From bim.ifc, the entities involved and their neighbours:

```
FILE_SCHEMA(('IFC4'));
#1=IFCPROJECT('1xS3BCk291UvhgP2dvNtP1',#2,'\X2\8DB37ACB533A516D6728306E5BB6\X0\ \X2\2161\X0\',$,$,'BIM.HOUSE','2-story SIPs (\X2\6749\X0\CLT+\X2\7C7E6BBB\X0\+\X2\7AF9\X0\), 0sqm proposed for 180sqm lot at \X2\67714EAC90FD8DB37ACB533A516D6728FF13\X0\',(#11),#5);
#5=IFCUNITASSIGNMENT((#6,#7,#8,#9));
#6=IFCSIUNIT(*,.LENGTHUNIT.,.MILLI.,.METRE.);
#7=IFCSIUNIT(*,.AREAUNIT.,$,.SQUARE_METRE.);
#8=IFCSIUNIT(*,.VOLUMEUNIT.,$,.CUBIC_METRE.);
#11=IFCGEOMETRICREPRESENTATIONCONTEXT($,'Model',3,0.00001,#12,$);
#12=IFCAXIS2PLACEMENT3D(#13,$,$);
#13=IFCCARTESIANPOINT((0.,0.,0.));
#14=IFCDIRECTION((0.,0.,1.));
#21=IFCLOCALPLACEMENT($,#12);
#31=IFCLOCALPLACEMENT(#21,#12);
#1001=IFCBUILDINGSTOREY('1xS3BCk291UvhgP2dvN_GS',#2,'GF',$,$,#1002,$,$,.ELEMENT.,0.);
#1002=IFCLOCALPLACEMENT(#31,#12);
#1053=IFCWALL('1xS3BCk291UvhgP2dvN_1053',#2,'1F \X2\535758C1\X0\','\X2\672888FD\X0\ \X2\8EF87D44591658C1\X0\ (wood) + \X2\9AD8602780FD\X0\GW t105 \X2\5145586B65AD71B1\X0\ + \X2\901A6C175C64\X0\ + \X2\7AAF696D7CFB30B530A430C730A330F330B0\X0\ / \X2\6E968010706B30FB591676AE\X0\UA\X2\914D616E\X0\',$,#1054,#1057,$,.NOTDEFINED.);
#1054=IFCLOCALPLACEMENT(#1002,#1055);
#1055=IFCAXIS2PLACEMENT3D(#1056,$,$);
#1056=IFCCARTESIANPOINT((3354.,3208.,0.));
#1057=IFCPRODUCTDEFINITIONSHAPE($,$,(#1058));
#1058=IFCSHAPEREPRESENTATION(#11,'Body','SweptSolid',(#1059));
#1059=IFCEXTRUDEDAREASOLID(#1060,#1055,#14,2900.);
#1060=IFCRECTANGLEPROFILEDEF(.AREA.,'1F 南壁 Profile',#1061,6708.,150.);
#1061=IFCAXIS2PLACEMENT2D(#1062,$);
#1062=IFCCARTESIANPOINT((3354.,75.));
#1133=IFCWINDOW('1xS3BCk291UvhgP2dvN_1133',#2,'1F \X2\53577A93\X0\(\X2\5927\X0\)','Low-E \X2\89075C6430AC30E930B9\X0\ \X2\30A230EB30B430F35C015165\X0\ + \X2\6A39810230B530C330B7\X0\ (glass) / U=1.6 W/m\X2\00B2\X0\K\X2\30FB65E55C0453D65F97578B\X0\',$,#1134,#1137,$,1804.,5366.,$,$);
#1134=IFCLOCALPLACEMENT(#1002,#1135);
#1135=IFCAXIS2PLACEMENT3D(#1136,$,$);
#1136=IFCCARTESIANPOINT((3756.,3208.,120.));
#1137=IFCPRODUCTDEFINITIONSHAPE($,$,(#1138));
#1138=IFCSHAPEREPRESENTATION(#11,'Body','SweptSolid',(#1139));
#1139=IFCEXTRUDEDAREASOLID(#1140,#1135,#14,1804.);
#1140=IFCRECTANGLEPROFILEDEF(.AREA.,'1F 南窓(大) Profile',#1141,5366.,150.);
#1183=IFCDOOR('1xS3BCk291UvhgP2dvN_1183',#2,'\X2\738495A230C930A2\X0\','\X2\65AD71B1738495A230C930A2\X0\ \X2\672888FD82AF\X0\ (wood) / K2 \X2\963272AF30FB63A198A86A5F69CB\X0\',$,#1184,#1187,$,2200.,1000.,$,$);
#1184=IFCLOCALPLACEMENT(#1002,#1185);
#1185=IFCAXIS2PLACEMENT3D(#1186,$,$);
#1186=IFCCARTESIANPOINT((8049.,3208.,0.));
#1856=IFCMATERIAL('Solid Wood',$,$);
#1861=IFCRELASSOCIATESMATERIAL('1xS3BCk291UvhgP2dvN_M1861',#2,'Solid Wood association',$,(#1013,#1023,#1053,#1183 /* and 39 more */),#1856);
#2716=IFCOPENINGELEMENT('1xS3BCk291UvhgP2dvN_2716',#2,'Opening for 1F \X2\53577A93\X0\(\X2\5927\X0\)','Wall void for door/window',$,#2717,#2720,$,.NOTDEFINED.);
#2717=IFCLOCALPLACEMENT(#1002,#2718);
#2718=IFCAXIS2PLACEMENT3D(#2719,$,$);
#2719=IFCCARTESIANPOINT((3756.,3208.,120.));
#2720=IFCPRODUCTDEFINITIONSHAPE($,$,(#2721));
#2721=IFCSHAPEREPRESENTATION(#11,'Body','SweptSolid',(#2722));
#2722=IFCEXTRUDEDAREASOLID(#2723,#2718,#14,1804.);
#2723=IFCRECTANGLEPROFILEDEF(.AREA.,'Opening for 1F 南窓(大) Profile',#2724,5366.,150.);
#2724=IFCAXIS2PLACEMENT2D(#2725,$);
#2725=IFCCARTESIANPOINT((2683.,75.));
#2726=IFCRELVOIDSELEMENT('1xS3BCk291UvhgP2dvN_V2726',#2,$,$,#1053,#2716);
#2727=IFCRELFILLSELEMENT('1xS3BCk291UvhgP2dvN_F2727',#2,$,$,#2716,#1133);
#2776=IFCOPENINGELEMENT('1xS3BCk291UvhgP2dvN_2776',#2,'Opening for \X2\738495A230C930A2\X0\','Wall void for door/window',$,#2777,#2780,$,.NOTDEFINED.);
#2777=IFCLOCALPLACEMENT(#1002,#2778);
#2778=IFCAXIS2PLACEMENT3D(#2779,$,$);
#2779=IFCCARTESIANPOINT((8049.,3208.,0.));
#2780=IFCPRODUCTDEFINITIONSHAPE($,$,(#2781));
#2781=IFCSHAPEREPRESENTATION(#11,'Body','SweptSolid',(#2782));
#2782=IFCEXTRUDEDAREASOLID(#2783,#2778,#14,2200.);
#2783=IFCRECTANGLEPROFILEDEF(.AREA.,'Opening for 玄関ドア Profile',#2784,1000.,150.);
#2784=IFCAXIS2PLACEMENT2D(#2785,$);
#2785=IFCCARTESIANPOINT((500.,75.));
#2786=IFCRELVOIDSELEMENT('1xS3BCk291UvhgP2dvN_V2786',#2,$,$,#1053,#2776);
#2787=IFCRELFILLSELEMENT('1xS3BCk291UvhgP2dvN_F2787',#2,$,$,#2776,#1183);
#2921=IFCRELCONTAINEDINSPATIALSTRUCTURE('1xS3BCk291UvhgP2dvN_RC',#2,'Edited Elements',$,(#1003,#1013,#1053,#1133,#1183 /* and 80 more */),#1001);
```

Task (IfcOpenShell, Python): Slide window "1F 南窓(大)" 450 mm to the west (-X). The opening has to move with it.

```python
import ifcopenshell
import ifcopenshell.api.geometry
import ifcopenshell.util.placement
import ifcopenshell.util.unit

model = ifcopenshell.open("bim.ifc")
unit_scale = ifcopenshell.util.unit.calculate_unit_scale(model)

window = model.by_guid("1xS3BCk291UvhgP2dvN_1133")
opening = window.FillsVoids[0].RelatingOpeningElement
wall = opening.VoidsElements[0].RelatingBuildingElement

wall_matrix = ifcopenshell.util.placement.get_local_placement(wall.ObjectPlacement)
shift = wall_matrix[:3, 0] * -0.45 / unit_scale
before = ifcopenshell.util.placement.get_local_placement(window.ObjectPlacement)[:3, 3].copy()

# The window is not placed relative to its opening, so move both.
for product in (opening, window):
    matrix = ifcopenshell.util.placement.get_local_placement(product.ObjectPlacement)
    matrix[:3, 3] += shift
    ifcopenshell.api.geometry.edit_object_placement(model, product=product, matrix=matrix, is_si=False)

after = ifcopenshell.util.placement.get_local_placement(window.ObjectPlacement)[:3, 3]
print("window moved by", (after - before).round(3) + 0.0)

model.write("bim_updated.ifc")
```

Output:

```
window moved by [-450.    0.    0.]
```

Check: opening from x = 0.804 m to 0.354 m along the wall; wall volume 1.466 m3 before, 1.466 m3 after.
